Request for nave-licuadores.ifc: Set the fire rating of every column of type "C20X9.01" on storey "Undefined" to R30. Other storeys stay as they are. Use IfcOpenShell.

First a look at what the model holds.

```python
import ifcopenshell
import ifcopenshell.util.element

model = ifcopenshell.open("nave-licuadores.ifc")
print(model.schema)
storey = next(s for s in model.by_type("IfcBuildingStorey") if s.Name == "Undefined")
columns = [e for e in ifcopenshell.util.element.get_decomposition(storey) if e.is_a("IfcColumn")]
seen = {}
for e in columns:
    element_type = ifcopenshell.util.element.get_type(e)
    key = (element_type.Name if element_type != e and element_type else None, ifcopenshell.util.element.get_pset(e, "Pset_ColumnCommon", "FireRating"))
    seen[key] = seen.get(key, 0) + 1
for (name, value), count in sorted(seen.items(), key=str):
    print(count, "x", name, "|", value)
```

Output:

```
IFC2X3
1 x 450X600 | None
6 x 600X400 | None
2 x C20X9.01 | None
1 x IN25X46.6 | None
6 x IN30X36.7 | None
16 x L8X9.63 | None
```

```python
import ifcopenshell
import ifcopenshell.api.pset
import ifcopenshell.util.element

model = ifcopenshell.open("nave-licuadores.ifc")

storey = next(s for s in model.by_type("IfcBuildingStorey") if s.Name == "Undefined")
columns = [e for e in ifcopenshell.util.element.get_decomposition(storey) if e.is_a("IfcColumn")]

count = 0
for e in columns:
    element_type = ifcopenshell.util.element.get_type(e)
    if element_type in (None, e) or element_type.Name != "C20X9.01":
        continue
    # add_pset returns the element's existing set when there is one.
    pset = ifcopenshell.api.pset.add_pset(model, product=e, name="Pset_ColumnCommon")
    ifcopenshell.api.pset.edit_pset(model, pset=pset, properties={"FireRating": "R30"})
    count += 1

print(count, "columns updated")

model.write("nave-licuadores_edited.ifc")
```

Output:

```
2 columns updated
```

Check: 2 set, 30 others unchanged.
